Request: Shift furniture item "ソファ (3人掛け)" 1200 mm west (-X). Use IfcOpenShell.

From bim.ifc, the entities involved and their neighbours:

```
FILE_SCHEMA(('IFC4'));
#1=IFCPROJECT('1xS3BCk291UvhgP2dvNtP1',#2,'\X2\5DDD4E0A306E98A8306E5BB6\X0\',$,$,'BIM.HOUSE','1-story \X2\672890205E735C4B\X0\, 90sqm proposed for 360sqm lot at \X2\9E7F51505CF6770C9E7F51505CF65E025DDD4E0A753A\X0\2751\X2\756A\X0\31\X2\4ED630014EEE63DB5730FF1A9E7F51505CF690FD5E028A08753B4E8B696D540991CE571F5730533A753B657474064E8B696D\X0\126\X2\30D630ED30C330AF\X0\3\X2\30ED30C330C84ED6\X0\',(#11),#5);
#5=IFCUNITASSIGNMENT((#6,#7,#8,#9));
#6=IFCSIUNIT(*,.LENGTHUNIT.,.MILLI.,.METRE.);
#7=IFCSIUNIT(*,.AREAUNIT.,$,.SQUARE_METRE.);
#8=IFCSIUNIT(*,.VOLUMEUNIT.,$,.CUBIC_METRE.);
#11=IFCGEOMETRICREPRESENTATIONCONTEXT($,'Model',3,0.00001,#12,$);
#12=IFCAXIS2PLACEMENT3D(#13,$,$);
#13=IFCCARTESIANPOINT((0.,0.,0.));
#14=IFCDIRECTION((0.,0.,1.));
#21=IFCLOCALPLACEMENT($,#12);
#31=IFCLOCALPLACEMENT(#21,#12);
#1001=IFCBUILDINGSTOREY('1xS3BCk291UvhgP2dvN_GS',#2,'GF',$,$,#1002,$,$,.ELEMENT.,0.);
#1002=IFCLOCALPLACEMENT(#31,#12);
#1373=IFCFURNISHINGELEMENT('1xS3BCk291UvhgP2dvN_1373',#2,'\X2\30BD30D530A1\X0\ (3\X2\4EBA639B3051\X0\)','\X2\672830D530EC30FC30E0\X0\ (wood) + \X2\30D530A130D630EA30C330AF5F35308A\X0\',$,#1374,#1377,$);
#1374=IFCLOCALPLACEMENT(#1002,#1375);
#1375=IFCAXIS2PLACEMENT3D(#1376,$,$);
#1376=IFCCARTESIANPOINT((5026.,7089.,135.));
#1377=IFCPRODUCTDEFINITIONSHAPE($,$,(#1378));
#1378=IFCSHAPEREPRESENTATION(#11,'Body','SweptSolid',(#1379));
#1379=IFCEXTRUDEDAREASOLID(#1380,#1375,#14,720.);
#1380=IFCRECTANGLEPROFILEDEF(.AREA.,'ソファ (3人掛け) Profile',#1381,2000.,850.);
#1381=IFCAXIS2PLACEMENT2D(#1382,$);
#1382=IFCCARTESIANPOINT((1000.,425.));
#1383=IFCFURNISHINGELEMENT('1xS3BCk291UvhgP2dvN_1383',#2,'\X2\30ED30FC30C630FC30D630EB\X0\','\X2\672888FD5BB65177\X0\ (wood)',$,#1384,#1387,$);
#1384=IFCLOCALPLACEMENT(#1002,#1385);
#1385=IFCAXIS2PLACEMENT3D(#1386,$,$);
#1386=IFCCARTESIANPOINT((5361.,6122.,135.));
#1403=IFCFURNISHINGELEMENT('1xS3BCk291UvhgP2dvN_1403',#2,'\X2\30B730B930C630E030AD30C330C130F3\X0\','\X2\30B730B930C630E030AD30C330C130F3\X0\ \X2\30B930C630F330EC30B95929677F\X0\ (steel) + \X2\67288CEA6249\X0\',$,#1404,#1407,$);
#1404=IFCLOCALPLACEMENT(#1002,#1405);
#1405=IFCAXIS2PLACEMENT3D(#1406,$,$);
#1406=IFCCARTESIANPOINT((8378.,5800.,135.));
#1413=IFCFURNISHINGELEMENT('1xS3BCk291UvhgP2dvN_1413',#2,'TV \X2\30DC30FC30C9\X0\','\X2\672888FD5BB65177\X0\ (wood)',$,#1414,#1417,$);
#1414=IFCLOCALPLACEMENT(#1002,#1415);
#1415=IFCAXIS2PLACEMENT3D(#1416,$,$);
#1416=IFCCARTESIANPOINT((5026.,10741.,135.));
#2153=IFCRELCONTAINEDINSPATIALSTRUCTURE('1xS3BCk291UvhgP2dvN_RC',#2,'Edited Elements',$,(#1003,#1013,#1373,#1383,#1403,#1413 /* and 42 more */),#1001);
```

```python
import ifcopenshell
import ifcopenshell.api.geometry
import ifcopenshell.util.placement
import ifcopenshell.util.unit

model = ifcopenshell.open("bim.ifc")
unit_scale = ifcopenshell.util.unit.calculate_unit_scale(model)

item = model.by_id(1373)
matrix = ifcopenshell.util.placement.get_local_placement(item.ObjectPlacement)
matrix[0, 3] -= 1.2 / unit_scale
ifcopenshell.api.geometry.edit_object_placement(model, product=item, matrix=matrix, is_si=False)

print(ifcopenshell.util.placement.get_local_placement(item.ObjectPlacement).round(3) + 0.0)

model.write("bim_v2.ifc")
```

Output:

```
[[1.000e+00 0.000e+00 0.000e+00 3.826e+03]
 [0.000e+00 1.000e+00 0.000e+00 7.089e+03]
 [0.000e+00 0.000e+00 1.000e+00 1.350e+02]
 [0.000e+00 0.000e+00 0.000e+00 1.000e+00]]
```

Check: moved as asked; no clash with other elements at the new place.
